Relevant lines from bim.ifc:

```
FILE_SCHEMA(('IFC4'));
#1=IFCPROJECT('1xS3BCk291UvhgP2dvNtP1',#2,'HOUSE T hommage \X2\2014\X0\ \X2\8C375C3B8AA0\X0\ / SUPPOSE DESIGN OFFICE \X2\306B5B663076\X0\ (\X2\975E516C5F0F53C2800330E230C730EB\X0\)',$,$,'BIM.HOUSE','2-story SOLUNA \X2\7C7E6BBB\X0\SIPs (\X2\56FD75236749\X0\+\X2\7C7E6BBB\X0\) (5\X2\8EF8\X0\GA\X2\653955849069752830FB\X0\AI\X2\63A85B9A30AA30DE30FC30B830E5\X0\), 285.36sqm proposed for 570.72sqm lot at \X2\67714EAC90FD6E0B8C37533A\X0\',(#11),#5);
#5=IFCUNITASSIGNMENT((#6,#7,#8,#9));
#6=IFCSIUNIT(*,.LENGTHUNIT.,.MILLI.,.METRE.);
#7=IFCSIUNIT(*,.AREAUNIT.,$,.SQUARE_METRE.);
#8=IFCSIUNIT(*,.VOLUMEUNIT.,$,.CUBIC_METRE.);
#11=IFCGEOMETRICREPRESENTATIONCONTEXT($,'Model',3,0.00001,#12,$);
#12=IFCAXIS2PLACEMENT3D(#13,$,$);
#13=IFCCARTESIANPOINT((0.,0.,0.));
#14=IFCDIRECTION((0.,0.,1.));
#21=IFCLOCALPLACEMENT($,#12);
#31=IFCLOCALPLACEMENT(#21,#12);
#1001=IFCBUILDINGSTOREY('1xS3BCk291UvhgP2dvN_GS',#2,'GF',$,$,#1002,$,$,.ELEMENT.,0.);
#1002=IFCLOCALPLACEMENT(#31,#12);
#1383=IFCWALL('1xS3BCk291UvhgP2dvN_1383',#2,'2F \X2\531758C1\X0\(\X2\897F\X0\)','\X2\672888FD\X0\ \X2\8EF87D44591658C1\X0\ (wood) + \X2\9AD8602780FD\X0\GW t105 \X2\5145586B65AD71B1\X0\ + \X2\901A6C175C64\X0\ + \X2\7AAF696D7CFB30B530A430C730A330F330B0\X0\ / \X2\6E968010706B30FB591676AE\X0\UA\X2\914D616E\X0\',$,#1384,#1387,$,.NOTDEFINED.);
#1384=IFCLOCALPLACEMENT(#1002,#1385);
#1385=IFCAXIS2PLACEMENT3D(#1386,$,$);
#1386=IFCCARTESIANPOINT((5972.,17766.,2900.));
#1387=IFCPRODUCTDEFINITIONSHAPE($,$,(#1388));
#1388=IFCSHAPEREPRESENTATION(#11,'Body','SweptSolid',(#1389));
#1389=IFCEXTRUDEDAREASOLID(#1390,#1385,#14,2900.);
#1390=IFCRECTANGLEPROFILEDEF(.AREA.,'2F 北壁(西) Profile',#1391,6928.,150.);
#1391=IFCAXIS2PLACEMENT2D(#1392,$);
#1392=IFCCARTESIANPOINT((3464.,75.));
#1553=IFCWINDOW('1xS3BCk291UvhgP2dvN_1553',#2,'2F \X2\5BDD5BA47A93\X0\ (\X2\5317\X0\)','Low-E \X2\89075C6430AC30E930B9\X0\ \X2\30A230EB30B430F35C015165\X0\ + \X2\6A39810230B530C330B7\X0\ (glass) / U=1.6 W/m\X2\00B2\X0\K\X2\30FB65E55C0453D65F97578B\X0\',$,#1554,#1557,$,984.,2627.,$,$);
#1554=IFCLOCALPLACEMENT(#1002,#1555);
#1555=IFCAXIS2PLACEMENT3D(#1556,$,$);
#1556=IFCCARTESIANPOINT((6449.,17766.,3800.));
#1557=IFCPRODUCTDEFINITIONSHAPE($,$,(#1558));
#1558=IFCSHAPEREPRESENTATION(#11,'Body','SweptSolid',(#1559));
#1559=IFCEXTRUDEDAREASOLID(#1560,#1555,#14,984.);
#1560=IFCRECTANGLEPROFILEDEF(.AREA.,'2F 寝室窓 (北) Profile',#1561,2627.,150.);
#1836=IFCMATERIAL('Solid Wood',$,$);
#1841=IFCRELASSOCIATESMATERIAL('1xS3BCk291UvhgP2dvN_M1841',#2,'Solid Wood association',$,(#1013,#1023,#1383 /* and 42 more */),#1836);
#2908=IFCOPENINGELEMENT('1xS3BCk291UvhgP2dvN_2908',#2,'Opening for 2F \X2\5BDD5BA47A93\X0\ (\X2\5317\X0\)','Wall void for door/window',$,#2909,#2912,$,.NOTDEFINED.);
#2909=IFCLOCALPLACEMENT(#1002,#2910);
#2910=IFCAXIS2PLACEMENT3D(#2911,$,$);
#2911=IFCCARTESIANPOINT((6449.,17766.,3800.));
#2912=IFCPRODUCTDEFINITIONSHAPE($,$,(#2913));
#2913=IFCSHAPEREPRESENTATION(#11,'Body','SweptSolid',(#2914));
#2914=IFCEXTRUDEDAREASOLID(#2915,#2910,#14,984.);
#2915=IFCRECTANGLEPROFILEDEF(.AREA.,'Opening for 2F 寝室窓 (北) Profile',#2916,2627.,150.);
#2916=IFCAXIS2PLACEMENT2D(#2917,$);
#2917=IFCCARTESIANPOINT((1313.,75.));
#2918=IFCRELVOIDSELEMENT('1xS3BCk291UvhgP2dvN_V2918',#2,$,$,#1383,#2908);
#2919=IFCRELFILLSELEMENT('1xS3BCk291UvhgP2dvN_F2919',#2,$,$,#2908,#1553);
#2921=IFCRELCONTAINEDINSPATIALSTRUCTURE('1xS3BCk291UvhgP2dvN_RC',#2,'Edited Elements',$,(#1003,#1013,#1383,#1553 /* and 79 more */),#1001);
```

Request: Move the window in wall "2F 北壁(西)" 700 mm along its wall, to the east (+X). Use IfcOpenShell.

```python
import ifcopenshell
import ifcopenshell.api.geometry
import ifcopenshell.util.placement
import ifcopenshell.util.unit

model = ifcopenshell.open("bim.ifc")
unit_scale = ifcopenshell.util.unit.calculate_unit_scale(model)

window = model.by_guid("1xS3BCk291UvhgP2dvN_1553")
opening = window.FillsVoids[0].RelatingOpeningElement
wall = opening.VoidsElements[0].RelatingBuildingElement

wall_matrix = ifcopenshell.util.placement.get_local_placement(wall.ObjectPlacement)
shift = wall_matrix[:3, 0] * 0.7 / unit_scale
before = ifcopenshell.util.placement.get_local_placement(window.ObjectPlacement)[:3, 3].copy()

# The window is not placed relative to its opening, so move both.
for product in (opening, window):
    matrix = ifcopenshell.util.placement.get_local_placement(product.ObjectPlacement)
    matrix[:3, 3] += shift
    ifcopenshell.api.geometry.edit_object_placement(model, product=product, matrix=matrix, is_si=False)

after = ifcopenshell.util.placement.get_local_placement(window.ObjectPlacement)[:3, 3]
print("window moved by", (after - before).round(3) + 0.0)

model.write("bim_updated.ifc")
```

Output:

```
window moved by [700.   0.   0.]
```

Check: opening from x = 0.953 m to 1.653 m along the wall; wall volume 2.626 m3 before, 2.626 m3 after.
